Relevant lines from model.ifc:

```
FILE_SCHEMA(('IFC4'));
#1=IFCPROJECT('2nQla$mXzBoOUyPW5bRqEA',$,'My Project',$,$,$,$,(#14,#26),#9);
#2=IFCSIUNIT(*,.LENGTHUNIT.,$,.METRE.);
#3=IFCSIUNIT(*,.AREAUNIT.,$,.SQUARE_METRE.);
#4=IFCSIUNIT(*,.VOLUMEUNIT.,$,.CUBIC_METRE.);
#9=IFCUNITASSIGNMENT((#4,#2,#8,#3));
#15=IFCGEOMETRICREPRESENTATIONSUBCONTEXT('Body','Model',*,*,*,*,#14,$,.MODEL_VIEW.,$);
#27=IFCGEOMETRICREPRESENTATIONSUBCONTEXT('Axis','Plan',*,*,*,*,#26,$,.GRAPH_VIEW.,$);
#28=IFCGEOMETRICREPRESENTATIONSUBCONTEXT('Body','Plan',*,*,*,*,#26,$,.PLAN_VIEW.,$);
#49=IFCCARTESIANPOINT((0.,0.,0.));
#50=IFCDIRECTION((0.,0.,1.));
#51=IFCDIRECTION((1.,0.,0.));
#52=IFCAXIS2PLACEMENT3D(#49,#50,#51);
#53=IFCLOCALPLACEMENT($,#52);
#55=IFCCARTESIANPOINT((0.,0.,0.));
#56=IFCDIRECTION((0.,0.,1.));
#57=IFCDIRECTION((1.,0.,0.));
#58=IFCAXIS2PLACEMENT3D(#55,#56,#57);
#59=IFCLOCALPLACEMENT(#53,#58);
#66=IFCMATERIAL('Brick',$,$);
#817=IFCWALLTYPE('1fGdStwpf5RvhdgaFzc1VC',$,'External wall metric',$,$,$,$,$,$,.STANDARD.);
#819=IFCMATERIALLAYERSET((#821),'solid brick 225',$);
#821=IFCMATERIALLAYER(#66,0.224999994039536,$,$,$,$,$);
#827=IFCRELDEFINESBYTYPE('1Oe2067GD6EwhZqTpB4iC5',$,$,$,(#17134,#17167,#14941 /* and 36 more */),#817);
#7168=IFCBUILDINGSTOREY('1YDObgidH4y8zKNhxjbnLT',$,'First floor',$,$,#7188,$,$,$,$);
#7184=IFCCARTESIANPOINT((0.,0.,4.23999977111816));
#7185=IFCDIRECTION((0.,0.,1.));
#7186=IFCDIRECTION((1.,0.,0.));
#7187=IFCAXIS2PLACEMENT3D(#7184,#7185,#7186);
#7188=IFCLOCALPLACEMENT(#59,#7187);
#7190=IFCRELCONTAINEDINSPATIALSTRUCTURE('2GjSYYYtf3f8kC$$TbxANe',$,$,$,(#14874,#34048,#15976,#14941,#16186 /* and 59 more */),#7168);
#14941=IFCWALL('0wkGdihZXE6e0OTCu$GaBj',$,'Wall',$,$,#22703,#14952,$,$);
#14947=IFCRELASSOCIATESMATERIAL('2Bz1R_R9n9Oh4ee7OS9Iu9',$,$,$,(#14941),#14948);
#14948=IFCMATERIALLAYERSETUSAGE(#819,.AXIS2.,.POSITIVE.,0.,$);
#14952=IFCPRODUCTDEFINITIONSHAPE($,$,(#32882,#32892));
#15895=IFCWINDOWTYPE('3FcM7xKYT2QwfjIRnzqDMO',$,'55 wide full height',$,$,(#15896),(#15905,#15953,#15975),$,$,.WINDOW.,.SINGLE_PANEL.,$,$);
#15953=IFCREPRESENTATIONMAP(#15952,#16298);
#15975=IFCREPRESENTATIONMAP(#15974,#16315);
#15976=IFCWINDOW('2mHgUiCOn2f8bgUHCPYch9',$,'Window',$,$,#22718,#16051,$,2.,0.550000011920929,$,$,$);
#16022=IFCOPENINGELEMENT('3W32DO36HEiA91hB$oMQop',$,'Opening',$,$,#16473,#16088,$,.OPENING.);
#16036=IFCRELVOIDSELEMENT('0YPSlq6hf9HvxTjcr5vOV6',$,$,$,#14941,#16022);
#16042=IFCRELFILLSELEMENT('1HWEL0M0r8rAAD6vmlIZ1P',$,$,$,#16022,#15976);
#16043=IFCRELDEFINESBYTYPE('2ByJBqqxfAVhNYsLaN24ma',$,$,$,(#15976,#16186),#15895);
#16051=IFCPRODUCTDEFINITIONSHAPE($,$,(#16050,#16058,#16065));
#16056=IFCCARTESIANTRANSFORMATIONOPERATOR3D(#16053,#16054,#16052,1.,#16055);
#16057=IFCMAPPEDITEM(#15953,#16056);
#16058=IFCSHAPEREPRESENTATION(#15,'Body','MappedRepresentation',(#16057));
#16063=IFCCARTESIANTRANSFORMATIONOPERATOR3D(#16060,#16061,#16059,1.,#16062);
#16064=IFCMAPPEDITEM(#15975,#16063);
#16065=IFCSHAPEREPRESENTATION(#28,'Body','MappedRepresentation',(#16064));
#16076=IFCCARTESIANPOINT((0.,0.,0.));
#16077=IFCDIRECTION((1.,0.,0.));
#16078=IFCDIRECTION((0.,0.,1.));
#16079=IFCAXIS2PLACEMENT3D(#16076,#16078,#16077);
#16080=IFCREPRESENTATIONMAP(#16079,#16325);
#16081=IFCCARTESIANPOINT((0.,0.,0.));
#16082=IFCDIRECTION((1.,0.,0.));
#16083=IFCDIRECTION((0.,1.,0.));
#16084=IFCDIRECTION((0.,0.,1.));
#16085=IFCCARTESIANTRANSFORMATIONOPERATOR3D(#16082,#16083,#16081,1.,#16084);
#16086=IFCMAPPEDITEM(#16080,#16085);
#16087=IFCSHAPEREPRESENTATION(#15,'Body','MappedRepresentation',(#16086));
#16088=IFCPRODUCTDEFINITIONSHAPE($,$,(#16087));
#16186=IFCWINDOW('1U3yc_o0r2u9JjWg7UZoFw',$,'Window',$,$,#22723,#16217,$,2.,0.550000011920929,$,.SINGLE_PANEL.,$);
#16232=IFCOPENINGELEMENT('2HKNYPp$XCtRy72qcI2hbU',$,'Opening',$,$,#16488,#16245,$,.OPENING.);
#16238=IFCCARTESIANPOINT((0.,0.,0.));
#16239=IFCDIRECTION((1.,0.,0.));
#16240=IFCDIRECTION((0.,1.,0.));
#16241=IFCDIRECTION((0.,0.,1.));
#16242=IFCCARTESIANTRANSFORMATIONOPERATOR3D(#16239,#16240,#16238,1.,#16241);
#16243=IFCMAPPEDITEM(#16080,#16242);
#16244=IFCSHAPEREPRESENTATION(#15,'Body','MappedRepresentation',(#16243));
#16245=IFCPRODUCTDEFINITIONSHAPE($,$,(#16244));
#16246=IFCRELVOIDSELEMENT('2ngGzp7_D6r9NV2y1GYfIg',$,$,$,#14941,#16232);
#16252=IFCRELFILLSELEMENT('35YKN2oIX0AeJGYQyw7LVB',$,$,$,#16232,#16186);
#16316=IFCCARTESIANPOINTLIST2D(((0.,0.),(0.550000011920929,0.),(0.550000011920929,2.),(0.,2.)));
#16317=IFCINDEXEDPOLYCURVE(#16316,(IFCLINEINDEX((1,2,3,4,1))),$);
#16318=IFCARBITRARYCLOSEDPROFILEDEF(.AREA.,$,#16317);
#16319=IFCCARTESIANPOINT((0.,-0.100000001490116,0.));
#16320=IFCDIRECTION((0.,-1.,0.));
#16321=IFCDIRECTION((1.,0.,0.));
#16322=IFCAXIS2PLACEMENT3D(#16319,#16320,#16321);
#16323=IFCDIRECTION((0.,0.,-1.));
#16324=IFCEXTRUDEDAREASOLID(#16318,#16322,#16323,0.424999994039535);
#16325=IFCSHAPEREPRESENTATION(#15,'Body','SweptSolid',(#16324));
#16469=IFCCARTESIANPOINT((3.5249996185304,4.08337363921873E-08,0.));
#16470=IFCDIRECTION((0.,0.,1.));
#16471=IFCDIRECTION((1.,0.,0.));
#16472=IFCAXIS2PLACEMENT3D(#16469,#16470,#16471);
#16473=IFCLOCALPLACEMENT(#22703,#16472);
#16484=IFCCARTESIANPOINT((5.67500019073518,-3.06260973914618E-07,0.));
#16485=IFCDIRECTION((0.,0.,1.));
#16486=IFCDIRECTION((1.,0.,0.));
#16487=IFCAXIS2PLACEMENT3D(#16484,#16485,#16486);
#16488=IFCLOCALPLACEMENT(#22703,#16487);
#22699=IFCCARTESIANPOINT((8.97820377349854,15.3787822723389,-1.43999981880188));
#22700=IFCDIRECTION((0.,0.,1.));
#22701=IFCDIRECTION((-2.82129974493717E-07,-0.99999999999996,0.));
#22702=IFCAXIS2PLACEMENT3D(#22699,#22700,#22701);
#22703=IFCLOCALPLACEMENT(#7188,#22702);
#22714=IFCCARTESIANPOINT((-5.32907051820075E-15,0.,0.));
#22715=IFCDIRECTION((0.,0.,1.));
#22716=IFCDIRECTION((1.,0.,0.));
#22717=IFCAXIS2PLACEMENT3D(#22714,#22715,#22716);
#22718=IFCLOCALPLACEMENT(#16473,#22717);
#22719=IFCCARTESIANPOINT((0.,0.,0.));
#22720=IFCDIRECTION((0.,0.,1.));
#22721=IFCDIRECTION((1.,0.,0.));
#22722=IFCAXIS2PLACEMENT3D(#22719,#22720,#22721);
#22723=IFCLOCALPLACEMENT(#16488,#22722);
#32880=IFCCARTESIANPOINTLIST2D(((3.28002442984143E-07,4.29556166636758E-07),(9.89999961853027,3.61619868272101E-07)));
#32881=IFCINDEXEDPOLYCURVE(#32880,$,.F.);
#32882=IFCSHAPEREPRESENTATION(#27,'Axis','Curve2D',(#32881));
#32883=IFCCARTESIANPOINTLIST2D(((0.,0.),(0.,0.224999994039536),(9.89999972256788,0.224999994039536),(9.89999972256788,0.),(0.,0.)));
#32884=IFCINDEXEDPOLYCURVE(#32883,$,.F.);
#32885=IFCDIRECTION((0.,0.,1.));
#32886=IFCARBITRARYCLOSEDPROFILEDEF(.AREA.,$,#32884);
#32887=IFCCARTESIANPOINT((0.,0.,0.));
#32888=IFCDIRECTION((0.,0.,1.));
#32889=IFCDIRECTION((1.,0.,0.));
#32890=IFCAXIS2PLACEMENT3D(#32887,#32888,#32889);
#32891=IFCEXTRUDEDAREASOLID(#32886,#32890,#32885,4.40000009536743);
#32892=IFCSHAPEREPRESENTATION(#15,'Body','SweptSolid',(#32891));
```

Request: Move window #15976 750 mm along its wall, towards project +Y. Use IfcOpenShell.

```python
import ifcopenshell
import ifcopenshell.api.geometry
import ifcopenshell.util.placement
import ifcopenshell.util.unit

model = ifcopenshell.open("model.ifc")
unit_scale = ifcopenshell.util.unit.calculate_unit_scale(model)

window = model.by_guid("2mHgUiCOn2f8bgUHCPYch9")
opening = window.FillsVoids[0].RelatingOpeningElement
wall = opening.VoidsElements[0].RelatingBuildingElement

wall_matrix = ifcopenshell.util.placement.get_local_placement(wall.ObjectPlacement)
shift = wall_matrix[:3, 0] * -0.75 / unit_scale
before = ifcopenshell.util.placement.get_local_placement(window.ObjectPlacement)[:3, 3].copy()

# The window is placed relative to its opening, so it follows when the opening moves.
matrix = ifcopenshell.util.placement.get_local_placement(opening.ObjectPlacement)
matrix[:3, 3] += shift
ifcopenshell.api.geometry.edit_object_placement(
    model, product=opening, matrix=matrix, is_si=False, should_transform_children=True
)

after = ifcopenshell.util.placement.get_local_placement(window.ObjectPlacement)[:3, 3]
print("window moved by", (after - before).round(3) + 0.0)

model.write("model_edited.ifc")
```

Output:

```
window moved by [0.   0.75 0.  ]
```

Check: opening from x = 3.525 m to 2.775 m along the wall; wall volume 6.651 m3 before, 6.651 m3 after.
